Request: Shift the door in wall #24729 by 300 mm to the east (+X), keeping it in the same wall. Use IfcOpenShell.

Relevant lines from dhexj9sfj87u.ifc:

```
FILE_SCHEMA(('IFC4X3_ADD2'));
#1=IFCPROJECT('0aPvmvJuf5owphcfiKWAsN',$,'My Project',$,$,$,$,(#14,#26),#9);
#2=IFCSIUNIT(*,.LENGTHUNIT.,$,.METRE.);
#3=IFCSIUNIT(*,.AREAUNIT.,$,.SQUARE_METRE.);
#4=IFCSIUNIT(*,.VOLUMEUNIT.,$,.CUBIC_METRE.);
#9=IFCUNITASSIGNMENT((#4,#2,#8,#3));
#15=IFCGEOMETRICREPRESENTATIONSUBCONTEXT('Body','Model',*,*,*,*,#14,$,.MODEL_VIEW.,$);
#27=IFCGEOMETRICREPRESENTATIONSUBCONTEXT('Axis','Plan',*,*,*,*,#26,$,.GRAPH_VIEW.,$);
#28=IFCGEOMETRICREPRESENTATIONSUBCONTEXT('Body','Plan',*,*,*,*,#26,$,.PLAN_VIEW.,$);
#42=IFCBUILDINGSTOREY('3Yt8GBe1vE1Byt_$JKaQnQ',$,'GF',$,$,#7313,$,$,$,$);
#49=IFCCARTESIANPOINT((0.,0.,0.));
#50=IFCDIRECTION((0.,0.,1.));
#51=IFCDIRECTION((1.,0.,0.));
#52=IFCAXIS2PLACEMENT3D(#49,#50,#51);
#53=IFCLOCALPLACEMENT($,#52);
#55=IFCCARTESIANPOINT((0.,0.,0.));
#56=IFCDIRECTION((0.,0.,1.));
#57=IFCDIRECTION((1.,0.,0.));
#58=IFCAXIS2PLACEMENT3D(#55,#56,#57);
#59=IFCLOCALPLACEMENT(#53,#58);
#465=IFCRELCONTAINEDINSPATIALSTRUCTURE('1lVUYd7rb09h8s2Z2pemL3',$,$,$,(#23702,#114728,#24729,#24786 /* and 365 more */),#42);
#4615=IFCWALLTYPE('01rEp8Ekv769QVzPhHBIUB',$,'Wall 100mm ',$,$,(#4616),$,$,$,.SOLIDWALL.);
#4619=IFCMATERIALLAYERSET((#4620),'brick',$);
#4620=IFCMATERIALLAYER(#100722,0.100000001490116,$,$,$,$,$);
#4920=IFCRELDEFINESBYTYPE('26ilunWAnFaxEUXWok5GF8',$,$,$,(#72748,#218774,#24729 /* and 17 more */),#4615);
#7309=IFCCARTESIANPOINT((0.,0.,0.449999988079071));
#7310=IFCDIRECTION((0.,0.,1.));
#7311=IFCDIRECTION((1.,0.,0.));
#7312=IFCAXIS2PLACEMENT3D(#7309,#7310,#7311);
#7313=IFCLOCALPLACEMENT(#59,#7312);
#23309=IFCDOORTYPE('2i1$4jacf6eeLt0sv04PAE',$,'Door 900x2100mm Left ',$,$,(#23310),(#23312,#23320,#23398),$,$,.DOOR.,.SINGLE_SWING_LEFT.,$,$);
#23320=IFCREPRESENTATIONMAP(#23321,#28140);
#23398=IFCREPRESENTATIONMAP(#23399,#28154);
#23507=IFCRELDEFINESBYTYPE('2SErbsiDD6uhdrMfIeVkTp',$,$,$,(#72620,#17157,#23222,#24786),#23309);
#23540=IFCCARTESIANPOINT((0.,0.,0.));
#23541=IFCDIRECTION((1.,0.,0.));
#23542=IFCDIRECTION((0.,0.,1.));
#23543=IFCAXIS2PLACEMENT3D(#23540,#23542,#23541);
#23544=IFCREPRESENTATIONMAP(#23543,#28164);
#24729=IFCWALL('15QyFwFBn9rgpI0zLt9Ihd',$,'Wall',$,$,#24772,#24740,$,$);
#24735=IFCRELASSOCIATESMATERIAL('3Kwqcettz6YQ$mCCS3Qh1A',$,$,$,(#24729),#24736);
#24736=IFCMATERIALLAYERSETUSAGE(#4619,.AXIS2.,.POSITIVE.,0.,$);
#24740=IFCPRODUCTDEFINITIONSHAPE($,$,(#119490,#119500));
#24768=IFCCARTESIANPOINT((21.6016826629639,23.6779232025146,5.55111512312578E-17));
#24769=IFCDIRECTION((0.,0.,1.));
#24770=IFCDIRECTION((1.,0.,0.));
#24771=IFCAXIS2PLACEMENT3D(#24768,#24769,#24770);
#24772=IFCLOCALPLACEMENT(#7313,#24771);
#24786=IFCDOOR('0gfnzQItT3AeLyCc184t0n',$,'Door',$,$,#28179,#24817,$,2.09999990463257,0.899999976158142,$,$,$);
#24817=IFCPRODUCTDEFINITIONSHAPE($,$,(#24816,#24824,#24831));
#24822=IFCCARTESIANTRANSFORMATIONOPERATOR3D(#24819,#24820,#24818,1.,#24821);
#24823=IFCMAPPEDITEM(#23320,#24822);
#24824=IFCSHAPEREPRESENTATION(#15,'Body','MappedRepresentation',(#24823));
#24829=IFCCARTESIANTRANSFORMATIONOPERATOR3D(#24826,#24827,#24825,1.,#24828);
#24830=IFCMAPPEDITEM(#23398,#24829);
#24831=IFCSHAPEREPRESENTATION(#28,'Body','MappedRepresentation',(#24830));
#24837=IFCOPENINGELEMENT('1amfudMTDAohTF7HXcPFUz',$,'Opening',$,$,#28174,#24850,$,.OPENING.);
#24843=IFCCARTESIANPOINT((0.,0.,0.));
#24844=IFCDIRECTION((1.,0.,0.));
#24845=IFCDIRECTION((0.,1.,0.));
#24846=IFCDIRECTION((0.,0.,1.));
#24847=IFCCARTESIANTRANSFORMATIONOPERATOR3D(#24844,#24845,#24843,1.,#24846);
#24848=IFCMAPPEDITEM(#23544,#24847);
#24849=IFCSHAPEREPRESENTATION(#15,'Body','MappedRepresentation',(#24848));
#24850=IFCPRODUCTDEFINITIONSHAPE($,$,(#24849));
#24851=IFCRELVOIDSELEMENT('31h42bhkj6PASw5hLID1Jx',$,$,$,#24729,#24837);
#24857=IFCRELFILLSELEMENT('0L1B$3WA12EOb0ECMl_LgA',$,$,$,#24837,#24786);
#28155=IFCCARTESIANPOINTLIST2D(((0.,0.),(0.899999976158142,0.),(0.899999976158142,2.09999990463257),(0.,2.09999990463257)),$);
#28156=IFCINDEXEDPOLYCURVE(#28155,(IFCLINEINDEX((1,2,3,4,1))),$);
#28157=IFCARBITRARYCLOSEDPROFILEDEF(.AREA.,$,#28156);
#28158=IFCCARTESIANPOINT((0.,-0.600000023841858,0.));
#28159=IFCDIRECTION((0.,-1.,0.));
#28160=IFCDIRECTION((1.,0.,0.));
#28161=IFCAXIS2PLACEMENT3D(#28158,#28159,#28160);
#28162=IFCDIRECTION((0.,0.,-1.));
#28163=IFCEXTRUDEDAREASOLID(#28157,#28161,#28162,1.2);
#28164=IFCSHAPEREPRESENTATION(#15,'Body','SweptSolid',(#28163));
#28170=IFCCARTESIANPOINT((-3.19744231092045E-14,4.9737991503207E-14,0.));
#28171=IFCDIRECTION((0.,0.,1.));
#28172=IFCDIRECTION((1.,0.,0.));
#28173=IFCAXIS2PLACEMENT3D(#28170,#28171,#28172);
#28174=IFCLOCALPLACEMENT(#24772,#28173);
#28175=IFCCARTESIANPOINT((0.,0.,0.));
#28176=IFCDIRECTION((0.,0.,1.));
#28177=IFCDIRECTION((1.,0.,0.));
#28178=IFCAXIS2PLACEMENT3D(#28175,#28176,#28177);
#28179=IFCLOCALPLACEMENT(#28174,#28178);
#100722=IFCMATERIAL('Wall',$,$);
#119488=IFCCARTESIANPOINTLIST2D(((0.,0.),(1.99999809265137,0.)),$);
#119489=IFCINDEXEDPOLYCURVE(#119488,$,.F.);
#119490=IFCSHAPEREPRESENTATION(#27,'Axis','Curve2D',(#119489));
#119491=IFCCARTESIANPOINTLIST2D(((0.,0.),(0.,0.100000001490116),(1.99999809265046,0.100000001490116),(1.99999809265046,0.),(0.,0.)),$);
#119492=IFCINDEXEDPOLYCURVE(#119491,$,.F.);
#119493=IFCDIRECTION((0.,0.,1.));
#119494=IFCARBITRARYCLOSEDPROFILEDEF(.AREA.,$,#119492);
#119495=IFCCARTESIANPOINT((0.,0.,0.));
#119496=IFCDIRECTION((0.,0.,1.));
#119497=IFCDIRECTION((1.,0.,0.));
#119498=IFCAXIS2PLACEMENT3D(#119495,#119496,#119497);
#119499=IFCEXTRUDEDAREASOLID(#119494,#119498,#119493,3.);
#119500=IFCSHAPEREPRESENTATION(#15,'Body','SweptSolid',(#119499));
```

```python
import ifcopenshell
import ifcopenshell.api.geometry
import ifcopenshell.util.placement

model = ifcopenshell.open("dhexj9sfj87u.ifc")

door = model.by_guid("0gfnzQItT3AeLyCc184t0n")
opening = door.FillsVoids[0].RelatingOpeningElement
wall = opening.VoidsElements[0].RelatingBuildingElement

wall_matrix = ifcopenshell.util.placement.get_local_placement(wall.ObjectPlacement)
shift = wall_matrix[:3, 0] * 0.3
before = ifcopenshell.util.placement.get_local_placement(door.ObjectPlacement)[:3, 3].copy()

# The door is placed relative to its opening, so it follows when the opening moves.
matrix = ifcopenshell.util.placement.get_local_placement(opening.ObjectPlacement)
matrix[:3, 3] += shift
ifcopenshell.api.geometry.edit_object_placement(
    model, product=opening, matrix=matrix, is_si=False, should_transform_children=True
)

after = ifcopenshell.util.placement.get_local_placement(door.ObjectPlacement)[:3, 3]
print("door moved by", (after - before).round(3) + 0.0)

model.write("dhexj9sfj87u_rev.ifc")
```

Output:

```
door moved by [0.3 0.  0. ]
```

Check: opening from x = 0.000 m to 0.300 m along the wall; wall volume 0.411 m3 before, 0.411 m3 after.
